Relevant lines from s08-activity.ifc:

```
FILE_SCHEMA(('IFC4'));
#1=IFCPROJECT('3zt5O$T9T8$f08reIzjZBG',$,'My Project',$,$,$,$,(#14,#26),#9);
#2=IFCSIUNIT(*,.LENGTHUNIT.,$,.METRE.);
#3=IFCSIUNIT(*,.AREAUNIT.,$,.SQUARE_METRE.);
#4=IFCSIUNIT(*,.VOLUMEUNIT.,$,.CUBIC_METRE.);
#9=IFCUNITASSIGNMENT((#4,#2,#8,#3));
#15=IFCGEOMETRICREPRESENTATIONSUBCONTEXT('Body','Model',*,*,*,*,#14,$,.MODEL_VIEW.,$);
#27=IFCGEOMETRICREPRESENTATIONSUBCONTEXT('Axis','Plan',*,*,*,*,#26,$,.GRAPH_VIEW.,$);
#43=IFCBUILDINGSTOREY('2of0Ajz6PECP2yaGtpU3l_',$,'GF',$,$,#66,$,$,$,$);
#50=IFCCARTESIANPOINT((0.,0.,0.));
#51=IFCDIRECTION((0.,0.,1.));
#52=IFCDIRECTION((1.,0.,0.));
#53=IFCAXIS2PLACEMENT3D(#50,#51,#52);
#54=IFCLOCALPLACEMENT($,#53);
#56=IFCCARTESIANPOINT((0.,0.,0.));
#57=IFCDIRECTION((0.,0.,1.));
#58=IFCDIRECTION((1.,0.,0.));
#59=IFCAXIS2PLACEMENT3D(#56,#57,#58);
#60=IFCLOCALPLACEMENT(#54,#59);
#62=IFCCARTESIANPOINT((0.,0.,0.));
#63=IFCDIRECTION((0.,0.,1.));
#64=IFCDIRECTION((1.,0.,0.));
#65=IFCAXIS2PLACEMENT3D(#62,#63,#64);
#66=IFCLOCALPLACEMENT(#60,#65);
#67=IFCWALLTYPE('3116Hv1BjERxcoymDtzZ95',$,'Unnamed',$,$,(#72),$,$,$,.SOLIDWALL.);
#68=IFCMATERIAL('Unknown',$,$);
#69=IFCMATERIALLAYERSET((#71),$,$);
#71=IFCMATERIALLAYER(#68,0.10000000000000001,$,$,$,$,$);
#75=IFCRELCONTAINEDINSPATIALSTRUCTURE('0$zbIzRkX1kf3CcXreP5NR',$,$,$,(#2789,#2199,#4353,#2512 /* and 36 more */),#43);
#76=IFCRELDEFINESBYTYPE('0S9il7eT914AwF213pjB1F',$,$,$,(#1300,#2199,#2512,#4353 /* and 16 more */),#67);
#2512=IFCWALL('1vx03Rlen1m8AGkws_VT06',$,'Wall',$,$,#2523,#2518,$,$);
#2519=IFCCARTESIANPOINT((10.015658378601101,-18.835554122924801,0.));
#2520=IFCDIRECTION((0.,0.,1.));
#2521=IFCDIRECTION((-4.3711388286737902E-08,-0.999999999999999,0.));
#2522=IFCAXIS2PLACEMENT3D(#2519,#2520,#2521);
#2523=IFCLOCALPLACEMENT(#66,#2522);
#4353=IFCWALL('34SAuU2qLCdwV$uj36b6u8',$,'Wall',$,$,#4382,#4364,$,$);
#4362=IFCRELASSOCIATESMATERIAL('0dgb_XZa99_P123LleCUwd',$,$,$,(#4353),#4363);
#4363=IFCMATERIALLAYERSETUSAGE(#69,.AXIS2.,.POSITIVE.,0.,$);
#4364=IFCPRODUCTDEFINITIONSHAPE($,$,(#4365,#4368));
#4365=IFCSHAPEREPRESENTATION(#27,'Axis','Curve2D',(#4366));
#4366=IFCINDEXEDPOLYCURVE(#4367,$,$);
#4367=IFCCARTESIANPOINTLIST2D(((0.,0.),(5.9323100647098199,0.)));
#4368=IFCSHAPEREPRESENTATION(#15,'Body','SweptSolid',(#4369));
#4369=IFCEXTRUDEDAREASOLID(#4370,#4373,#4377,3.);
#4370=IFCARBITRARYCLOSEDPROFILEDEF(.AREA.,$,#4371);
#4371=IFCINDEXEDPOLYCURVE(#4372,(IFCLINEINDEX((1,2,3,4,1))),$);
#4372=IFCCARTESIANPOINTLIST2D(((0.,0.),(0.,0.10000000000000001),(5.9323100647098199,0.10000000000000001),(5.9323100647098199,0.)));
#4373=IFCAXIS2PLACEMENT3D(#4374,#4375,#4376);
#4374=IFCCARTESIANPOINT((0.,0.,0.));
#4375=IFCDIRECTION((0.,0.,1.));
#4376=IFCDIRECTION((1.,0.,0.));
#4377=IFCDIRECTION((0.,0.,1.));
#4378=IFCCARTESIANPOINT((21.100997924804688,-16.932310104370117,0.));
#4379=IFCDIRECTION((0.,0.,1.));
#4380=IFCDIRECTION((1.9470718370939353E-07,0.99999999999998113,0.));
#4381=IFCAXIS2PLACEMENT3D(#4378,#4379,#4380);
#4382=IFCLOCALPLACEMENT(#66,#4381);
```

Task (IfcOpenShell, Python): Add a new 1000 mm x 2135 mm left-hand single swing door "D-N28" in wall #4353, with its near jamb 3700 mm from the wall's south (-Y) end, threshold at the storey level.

```python
import numpy as np
import ifcopenshell
import ifcopenshell.api.feature
import ifcopenshell.api.geometry
import ifcopenshell.api.root
import ifcopenshell.api.spatial
import ifcopenshell.geom
import ifcopenshell.util.element
import ifcopenshell.util.placement
import ifcopenshell.util.representation
import ifcopenshell.util.shape
import ifcopenshell.util.unit

model = ifcopenshell.open("s08-activity.ifc")
unit_scale = ifcopenshell.util.unit.calculate_unit_scale(model)
settings = ifcopenshell.geom.settings()


def volume(element):
    """Net volume in cubic metres, openings subtracted."""
    shape = ifcopenshell.geom.create_shape(settings, element)
    return ifcopenshell.util.shape.get_volume(shape.geometry)


wall = model.by_id(4353)
storey = ifcopenshell.util.element.get_container(wall, ifc_class="IfcBuildingStorey")
context = ifcopenshell.util.representation.get_context(model, "Model", "Body", "MODEL_VIEW")
before = volume(wall)

width, height, from_end, sill = 1, 2.135, 3.7, 0.0  # metres

# The wall runs along its own X axis, and the end named is its -X end.
wall_shape = ifcopenshell.geom.create_shape(settings, wall)
x, y, z = ifcopenshell.util.shape.get_vertices(wall_shape.geometry).T
start = x.min() + from_end
face, thickness = float(y.min()), float(y.max() - y.min())
wall_matrix = ifcopenshell.util.placement.get_local_placement(wall.ObjectPlacement)
level = ifcopenshell.util.placement.get_local_placement(storey.ObjectPlacement)[2, 3]


def in_wall(x, y):
    """Placement at x, y metres in the wall's axes, at sill height."""
    matrix = wall_matrix.copy()
    matrix[:, 3] = wall_matrix @ np.array([x / unit_scale, y / unit_scale, 0.0, 1.0])
    matrix[2, 3] = level + sill / unit_scale
    return matrix


# Opening: a box that overshoots both wall faces by 50 mm.
opening = ifcopenshell.api.root.create_entity(model, ifc_class="IfcOpeningElement", predefined_type="OPENING")
box = ifcopenshell.api.geometry.add_wall_representation(
    model, context=context, length=width, height=height, thickness=thickness + 0.1
)
ifcopenshell.api.geometry.assign_representation(model, product=opening, representation=box)
ifcopenshell.api.geometry.edit_object_placement(model, product=opening, matrix=in_wall(start, face - 0.05), is_si=False)
ifcopenshell.api.feature.add_feature(model, feature=opening, element=wall)

door = ifcopenshell.api.root.create_entity(model, ifc_class="IfcDoor", name="D-N28", predefined_type="DOOR")
door.OverallWidth, door.OverallHeight = width / unit_scale, height / unit_scale
door.OperationType = "SINGLE_SWING_LEFT"
body = ifcopenshell.api.geometry.add_door_representation(
    model,
    context=context,
    overall_width=door.OverallWidth,
    overall_height=door.OverallHeight,
    operation_type="SINGLE_SWING_LEFT",
    lining_properties={"LiningDepth": thickness / unit_scale, "ThresholdDepth": thickness / unit_scale},
)
ifcopenshell.api.geometry.assign_representation(model, product=door, representation=body)
ifcopenshell.api.spatial.assign_container(model, products=[door], relating_structure=storey)
ifcopenshell.api.feature.add_filling(model, opening=opening, element=door)

# The lining spans the wall, so the door starts at the wall face.
ifcopenshell.api.geometry.edit_object_placement(model, product=door, matrix=in_wall(start, face), is_si=False)

after = volume(wall)

print(f"wall volume {before:.3f} -> {after:.3f} m3")

model.write("s08-activity_updated.ifc")
```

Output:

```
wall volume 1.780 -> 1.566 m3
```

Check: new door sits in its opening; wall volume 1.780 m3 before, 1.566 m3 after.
